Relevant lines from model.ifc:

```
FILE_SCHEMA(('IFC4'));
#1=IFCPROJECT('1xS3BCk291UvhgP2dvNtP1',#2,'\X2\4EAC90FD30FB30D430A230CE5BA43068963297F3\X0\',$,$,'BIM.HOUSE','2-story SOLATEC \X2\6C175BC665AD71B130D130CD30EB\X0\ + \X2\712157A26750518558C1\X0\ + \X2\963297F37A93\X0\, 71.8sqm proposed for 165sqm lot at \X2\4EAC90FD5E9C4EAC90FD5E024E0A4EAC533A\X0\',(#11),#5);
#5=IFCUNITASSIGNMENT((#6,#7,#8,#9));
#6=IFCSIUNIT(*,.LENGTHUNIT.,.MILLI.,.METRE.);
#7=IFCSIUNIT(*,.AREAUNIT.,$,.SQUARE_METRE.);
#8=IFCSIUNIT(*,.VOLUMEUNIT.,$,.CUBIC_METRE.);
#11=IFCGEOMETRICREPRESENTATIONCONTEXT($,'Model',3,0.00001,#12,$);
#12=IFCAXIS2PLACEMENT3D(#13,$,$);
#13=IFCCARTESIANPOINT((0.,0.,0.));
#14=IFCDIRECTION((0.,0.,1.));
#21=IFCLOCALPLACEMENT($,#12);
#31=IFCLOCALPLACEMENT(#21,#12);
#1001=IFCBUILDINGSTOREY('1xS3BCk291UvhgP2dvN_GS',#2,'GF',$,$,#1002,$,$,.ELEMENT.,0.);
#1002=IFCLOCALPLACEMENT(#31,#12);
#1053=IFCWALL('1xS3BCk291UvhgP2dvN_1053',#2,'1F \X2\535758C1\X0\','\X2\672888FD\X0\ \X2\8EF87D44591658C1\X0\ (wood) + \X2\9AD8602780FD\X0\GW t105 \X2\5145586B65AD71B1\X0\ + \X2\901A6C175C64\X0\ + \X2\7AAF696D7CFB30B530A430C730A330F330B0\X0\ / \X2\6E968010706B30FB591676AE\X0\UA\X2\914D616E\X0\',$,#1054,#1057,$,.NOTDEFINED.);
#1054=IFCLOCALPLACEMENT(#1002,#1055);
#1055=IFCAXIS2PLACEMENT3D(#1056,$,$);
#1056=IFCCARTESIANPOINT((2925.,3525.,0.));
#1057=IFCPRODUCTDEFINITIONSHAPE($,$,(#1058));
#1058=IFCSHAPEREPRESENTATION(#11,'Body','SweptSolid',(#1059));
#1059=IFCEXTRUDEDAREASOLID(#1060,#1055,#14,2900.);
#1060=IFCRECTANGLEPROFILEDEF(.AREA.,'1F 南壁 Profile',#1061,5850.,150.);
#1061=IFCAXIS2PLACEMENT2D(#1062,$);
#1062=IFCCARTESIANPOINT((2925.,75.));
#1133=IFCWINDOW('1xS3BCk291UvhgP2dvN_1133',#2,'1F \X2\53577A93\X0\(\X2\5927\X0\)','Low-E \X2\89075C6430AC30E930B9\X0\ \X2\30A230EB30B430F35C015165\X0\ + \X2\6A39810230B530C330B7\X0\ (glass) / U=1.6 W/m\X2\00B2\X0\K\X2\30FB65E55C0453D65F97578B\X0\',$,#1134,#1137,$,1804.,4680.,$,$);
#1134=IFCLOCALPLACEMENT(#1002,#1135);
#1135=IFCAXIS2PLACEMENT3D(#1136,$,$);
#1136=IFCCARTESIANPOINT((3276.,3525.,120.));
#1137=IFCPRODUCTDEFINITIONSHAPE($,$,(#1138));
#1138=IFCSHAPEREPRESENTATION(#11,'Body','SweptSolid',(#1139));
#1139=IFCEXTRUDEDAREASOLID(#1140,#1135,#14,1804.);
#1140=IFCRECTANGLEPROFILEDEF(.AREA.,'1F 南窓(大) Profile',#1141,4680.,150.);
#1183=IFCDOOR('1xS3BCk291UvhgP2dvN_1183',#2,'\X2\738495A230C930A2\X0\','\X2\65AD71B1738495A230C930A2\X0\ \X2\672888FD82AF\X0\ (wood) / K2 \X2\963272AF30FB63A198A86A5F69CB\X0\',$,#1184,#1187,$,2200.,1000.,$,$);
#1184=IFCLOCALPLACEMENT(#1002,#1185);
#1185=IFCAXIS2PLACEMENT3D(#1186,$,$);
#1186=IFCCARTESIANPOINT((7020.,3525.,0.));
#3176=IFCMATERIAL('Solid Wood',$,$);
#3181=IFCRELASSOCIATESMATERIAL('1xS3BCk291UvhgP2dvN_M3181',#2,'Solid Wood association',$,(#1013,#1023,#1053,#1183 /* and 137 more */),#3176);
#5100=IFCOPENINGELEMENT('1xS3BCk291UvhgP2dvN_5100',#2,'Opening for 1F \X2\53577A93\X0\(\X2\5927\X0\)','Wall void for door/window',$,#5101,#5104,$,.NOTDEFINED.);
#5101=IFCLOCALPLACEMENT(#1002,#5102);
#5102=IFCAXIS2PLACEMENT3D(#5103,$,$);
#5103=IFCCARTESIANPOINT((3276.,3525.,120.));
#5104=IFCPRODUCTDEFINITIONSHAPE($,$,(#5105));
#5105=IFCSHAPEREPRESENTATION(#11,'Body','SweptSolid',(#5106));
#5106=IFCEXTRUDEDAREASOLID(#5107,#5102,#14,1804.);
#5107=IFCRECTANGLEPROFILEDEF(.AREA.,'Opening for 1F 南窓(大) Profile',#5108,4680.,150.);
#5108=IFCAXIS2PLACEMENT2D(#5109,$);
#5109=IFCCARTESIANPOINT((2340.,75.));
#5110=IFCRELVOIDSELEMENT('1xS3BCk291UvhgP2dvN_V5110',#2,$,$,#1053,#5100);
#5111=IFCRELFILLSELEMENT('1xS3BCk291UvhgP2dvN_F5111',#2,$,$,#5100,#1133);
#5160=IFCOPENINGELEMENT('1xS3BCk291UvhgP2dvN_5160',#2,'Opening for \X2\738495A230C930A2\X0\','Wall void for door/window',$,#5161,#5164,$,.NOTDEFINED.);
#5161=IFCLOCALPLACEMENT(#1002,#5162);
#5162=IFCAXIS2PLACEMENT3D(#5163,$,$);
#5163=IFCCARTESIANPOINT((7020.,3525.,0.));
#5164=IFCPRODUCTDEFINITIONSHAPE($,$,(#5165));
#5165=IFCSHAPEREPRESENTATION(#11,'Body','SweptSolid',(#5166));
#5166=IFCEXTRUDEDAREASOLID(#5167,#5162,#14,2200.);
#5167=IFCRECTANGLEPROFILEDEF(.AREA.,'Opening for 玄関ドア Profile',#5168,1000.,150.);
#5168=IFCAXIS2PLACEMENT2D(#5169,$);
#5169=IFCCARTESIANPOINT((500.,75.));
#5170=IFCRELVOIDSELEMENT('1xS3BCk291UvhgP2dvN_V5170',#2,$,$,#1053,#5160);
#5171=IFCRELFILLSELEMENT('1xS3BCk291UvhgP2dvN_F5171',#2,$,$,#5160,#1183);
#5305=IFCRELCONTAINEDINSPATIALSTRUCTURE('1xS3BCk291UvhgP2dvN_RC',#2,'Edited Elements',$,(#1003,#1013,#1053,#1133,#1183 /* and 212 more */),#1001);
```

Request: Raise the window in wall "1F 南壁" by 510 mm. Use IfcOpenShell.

```python
import numpy as np
import ifcopenshell
import ifcopenshell.api.geometry
import ifcopenshell.util.placement
import ifcopenshell.util.unit

model = ifcopenshell.open("model.ifc")
unit_scale = ifcopenshell.util.unit.calculate_unit_scale(model)

window = model.by_guid("1xS3BCk291UvhgP2dvN_1133")
opening = window.FillsVoids[0].RelatingOpeningElement
dz = 0.51 / unit_scale

shift = np.array([0.0, 0.0, dz])
# The window is not placed relative to its opening, so move both.
for product in (opening, window):
    matrix = ifcopenshell.util.placement.get_local_placement(product.ObjectPlacement)
    matrix[:3, 3] += shift
    ifcopenshell.api.geometry.edit_object_placement(model, product=product, matrix=matrix, is_si=False)

print(f"moved by {dz * unit_scale:+.3f} m")

model.write("model_edited.ifc")
```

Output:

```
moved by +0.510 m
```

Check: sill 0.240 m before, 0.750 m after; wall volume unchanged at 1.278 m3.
